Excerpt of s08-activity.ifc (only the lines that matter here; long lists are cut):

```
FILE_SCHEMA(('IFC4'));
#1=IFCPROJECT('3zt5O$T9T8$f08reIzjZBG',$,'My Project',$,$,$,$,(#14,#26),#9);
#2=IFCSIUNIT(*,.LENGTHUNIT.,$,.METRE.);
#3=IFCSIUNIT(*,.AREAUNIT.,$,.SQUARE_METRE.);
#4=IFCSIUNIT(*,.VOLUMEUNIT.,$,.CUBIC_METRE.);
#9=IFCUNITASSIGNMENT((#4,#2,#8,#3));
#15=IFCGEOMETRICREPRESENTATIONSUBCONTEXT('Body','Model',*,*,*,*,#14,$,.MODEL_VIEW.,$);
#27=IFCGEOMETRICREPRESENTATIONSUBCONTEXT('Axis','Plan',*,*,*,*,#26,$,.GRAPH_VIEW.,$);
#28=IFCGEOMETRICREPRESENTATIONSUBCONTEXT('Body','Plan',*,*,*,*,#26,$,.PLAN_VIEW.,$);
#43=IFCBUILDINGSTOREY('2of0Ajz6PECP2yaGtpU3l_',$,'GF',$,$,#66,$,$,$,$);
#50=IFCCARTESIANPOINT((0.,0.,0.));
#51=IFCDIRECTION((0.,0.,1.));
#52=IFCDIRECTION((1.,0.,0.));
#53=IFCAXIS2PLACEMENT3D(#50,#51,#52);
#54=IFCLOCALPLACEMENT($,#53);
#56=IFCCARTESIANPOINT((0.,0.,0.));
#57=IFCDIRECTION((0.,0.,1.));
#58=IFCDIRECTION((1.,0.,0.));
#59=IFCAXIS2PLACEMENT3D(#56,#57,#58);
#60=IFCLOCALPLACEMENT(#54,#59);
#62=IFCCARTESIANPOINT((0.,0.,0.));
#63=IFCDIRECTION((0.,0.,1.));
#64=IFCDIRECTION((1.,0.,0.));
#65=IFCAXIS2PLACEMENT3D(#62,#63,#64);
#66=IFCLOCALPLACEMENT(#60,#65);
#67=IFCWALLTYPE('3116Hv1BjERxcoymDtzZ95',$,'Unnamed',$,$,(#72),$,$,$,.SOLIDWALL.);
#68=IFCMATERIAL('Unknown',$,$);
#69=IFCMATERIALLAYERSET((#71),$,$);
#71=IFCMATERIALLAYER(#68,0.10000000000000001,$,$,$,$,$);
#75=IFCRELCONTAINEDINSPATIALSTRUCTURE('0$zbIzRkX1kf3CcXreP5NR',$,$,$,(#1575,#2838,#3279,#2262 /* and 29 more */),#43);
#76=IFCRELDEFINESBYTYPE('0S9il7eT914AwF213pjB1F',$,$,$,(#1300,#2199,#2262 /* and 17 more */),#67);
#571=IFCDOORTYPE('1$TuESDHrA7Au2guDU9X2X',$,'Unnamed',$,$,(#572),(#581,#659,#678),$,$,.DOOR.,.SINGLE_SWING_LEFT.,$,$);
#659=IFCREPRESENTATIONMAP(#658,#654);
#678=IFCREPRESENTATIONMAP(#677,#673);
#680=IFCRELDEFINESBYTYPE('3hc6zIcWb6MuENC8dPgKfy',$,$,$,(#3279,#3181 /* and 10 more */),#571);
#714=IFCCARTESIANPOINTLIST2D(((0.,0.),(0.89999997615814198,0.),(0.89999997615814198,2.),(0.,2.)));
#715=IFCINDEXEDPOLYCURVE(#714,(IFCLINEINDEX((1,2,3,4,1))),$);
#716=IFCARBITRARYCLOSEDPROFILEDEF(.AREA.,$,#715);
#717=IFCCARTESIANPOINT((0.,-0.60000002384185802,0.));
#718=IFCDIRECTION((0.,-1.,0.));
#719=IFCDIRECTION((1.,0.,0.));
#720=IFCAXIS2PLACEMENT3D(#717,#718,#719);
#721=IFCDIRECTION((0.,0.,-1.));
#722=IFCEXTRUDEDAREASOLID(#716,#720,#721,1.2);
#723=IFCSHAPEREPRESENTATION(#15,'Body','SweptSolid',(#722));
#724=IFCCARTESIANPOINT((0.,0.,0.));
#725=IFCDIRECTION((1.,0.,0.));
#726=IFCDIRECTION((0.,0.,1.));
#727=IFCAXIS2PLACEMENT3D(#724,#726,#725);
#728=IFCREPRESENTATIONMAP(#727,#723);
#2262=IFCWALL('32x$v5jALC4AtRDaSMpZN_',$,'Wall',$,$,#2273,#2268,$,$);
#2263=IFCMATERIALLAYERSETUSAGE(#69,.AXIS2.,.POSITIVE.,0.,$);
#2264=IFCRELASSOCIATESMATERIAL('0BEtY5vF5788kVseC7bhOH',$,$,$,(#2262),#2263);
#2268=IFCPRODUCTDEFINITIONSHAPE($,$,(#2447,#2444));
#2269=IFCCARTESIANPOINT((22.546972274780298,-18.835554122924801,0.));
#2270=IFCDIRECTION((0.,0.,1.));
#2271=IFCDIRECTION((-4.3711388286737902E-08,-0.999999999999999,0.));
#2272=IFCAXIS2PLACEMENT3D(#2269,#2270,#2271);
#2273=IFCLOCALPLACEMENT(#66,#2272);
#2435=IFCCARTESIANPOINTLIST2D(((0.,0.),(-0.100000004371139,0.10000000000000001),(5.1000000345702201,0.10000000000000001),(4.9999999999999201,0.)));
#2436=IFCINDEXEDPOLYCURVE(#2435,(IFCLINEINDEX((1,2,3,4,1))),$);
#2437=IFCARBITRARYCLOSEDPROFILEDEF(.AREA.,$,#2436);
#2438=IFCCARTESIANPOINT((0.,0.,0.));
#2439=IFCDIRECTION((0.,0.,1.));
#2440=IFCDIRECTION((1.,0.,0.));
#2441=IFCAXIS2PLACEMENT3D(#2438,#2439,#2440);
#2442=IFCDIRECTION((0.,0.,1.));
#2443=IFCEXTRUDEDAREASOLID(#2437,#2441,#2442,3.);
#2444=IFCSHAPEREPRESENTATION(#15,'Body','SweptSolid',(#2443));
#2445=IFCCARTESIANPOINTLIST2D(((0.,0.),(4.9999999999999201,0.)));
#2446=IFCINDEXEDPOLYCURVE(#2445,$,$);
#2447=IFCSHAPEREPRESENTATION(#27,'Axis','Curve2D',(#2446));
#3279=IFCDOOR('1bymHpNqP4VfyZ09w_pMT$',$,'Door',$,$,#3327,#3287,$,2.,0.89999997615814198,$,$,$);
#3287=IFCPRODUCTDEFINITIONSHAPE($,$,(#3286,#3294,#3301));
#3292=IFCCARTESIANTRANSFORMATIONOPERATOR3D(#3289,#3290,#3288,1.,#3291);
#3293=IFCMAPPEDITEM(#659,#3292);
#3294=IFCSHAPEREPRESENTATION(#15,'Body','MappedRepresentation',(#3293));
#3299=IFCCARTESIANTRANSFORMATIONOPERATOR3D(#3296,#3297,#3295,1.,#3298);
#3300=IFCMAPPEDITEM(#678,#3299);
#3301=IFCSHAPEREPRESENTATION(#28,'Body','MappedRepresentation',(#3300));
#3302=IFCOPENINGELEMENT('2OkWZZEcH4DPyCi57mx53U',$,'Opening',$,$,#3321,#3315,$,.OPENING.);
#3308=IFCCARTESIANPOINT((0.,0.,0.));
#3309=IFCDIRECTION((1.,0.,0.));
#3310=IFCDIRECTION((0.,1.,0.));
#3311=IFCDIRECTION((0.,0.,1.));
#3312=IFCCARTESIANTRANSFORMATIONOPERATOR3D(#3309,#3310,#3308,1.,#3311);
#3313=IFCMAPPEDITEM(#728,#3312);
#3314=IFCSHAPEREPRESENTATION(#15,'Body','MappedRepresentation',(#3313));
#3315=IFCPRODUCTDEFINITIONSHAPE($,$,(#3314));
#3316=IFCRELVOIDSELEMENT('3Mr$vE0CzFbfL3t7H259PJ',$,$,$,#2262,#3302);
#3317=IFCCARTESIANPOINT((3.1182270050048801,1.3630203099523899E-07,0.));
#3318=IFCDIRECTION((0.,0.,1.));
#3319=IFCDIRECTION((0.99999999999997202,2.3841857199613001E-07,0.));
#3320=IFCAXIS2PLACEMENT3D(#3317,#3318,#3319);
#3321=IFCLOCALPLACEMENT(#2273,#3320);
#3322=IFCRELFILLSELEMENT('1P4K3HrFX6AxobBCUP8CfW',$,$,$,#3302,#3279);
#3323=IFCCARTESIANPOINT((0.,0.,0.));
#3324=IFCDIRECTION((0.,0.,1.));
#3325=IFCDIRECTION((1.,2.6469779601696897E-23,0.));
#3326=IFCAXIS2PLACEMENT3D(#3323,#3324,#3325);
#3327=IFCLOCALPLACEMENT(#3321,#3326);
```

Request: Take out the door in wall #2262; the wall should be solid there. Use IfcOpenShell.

```python
import ifcopenshell
import ifcopenshell.api.feature
import ifcopenshell.api.root
import ifcopenshell.geom
import ifcopenshell.util.shape

model = ifcopenshell.open("s08-activity.ifc")
settings = ifcopenshell.geom.settings()


def volume(element):
    """Net volume in cubic metres, openings subtracted."""
    shape = ifcopenshell.geom.create_shape(settings, element)
    return ifcopenshell.util.shape.get_volume(shape.geometry)


door = model.by_id(3279)
opening = door.FillsVoids[0].RelatingOpeningElement
wall = opening.VoidsElements[0].RelatingBuildingElement
before = volume(wall)

ifcopenshell.api.root.remove_product(model, product=door)
ifcopenshell.api.feature.remove_feature(model, feature=opening)

after = volume(wall)

print(f"wall volume {before:.3f} -> {after:.3f} m3")

model.write("s08-activity-out.ifc")
```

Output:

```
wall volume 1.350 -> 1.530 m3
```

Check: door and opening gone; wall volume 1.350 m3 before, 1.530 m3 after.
